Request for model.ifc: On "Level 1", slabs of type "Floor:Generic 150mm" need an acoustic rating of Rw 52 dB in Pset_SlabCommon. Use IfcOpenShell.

First a look at what the model holds.

```python
import ifcopenshell
import ifcopenshell.util.element

model = ifcopenshell.open("model.ifc")
print(model.schema)
storey = next(s for s in model.by_type("IfcBuildingStorey") if s.Name == "Level 1")
slabs = [e for e in ifcopenshell.util.element.get_decomposition(storey) if e.is_a("IfcSlab")]
seen = {}
for e in slabs:
    element_type = ifcopenshell.util.element.get_type(e)
    key = (element_type.Name if element_type != e and element_type else None, ifcopenshell.util.element.get_pset(e, "Pset_SlabCommon", "AcousticRating"))
    seen[key] = seen.get(key, 0) + 1
for (name, value), count in sorted(seen.items(), key=str):
    print(count, "x", name, "|", value)
```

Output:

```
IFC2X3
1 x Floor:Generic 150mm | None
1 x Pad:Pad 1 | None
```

```python
import ifcopenshell
import ifcopenshell.api.pset
import ifcopenshell.util.element

model = ifcopenshell.open("model.ifc")

storey = next(s for s in model.by_type("IfcBuildingStorey") if s.Name == "Level 1")
slabs = [e for e in ifcopenshell.util.element.get_decomposition(storey) if e.is_a("IfcSlab")]

count = 0
for e in slabs:
    element_type = ifcopenshell.util.element.get_type(e)
    if element_type in (None, e) or element_type.Name != "Floor:Generic 150mm":
        continue
    # add_pset returns the element's existing set when there is one.
    pset = ifcopenshell.api.pset.add_pset(model, product=e, name="Pset_SlabCommon")
    ifcopenshell.api.pset.edit_pset(model, pset=pset, properties={"AcousticRating": "Rw 52 dB"})
    count += 1

print(count, "slabs updated")

model.write("model_v2.ifc")
```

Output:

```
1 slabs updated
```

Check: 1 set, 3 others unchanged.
